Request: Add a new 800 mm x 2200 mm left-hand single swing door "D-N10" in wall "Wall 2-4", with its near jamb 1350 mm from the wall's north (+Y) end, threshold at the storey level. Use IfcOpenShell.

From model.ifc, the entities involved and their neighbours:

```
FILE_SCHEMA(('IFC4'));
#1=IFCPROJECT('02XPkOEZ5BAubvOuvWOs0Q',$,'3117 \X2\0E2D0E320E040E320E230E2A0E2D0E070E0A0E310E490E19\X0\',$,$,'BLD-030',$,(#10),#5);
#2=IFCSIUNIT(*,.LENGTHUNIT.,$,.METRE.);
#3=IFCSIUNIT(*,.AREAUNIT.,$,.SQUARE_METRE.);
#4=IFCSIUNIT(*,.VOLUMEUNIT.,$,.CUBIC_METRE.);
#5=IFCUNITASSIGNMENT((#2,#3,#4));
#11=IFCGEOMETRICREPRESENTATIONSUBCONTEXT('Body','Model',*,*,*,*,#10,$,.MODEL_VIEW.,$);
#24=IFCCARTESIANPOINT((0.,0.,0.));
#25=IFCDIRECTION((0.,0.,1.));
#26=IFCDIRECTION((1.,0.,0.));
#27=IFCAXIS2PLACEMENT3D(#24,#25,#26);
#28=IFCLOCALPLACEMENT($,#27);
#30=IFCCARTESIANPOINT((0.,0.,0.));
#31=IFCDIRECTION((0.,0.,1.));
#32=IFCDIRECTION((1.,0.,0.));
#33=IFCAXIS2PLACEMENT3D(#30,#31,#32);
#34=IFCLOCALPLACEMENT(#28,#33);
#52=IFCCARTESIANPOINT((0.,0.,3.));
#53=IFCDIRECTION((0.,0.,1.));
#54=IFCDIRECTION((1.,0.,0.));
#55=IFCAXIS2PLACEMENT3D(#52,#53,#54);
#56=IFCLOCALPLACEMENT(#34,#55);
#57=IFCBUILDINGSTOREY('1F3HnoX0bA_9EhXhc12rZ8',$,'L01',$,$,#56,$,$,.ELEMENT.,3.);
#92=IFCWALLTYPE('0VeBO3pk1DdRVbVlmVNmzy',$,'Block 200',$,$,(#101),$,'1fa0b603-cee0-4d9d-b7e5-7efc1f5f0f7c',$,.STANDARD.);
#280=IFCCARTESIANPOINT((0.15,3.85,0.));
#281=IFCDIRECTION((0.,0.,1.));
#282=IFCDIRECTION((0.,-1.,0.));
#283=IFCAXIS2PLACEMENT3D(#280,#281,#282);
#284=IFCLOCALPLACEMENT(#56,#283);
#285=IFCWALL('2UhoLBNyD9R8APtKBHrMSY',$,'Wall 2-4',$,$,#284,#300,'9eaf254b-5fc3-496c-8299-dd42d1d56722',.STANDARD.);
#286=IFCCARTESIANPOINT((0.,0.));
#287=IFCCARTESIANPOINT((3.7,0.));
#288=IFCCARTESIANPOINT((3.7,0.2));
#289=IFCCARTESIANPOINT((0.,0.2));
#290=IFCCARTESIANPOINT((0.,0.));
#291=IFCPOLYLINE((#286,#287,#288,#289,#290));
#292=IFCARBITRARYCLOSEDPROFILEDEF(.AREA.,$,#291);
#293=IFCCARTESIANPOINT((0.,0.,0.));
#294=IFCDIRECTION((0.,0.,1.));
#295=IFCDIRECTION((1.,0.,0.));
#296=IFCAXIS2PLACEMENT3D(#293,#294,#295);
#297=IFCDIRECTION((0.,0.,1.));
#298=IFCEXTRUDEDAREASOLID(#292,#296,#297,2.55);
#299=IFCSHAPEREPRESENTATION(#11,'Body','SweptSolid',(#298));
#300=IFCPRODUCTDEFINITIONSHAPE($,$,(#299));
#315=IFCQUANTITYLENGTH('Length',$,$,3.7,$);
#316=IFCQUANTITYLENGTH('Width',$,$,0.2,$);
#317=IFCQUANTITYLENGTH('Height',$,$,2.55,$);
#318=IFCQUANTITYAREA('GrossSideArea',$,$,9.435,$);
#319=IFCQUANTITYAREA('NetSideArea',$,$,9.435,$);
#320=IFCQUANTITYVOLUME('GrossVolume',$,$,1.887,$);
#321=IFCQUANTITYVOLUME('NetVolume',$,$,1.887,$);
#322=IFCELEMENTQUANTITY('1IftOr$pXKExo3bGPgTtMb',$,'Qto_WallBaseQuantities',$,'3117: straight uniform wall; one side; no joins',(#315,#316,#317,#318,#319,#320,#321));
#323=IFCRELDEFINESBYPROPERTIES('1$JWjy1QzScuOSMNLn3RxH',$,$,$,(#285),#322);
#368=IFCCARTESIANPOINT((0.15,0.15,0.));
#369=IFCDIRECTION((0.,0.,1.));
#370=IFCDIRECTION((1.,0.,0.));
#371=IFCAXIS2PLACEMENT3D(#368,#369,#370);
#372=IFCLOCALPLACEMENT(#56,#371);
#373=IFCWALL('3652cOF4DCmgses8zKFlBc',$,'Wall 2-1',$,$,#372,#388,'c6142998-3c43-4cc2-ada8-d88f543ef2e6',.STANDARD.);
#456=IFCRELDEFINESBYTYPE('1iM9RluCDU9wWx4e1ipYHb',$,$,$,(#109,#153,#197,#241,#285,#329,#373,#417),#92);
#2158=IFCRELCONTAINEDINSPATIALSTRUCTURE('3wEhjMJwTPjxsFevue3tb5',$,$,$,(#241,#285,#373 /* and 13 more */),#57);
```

```python
import numpy as np
import ifcopenshell
import ifcopenshell.api.feature
import ifcopenshell.api.geometry
import ifcopenshell.api.pset
import ifcopenshell.api.root
import ifcopenshell.api.spatial
import ifcopenshell.geom
import ifcopenshell.util.element
import ifcopenshell.util.placement
import ifcopenshell.util.representation
import ifcopenshell.util.shape
import ifcopenshell.util.unit

model = ifcopenshell.open("model.ifc")
unit_scale = ifcopenshell.util.unit.calculate_unit_scale(model)
area_scale = ifcopenshell.util.unit.calculate_unit_scale(model, "AREAUNIT")
volume_scale = ifcopenshell.util.unit.calculate_unit_scale(model, "VOLUMEUNIT")
settings = ifcopenshell.geom.settings()


def volume(element):
    """Net volume in cubic metres, openings subtracted."""
    shape = ifcopenshell.geom.create_shape(settings, element)
    return ifcopenshell.util.shape.get_volume(shape.geometry)


wall = model.by_guid("2UhoLBNyD9R8APtKBHrMSY")
storey = ifcopenshell.util.element.get_container(wall, ifc_class="IfcBuildingStorey")
context = ifcopenshell.util.representation.get_context(model, "Model", "Body", "MODEL_VIEW")
before = volume(wall)

width, height, from_end, sill = 0.8, 2.2, 1.35, 0.0  # metres

# The wall runs along its own X axis, and the end named is its -X end.
wall_shape = ifcopenshell.geom.create_shape(settings, wall)
x, y, z = ifcopenshell.util.shape.get_vertices(wall_shape.geometry).T
start = x.min() + from_end
face, thickness = float(y.min()), float(y.max() - y.min())
wall_matrix = ifcopenshell.util.placement.get_local_placement(wall.ObjectPlacement)
level = ifcopenshell.util.placement.get_local_placement(storey.ObjectPlacement)[2, 3]


def in_wall(x, y):
    """Placement at x, y metres in the wall's axes, at sill height."""
    matrix = wall_matrix.copy()
    matrix[:, 3] = wall_matrix @ np.array([x / unit_scale, y / unit_scale, 0.0, 1.0])
    matrix[2, 3] = level + sill / unit_scale
    return matrix


# Opening: a box that overshoots both wall faces by 50 mm.
opening = ifcopenshell.api.root.create_entity(model, ifc_class="IfcOpeningElement", predefined_type="OPENING")
box = ifcopenshell.api.geometry.add_wall_representation(
    model, context=context, length=width, height=height, thickness=thickness + 0.1
)
ifcopenshell.api.geometry.assign_representation(model, product=opening, representation=box)
ifcopenshell.api.geometry.edit_object_placement(model, product=opening, matrix=in_wall(start, face - 0.05), is_si=False)
ifcopenshell.api.feature.add_feature(model, feature=opening, element=wall)

door = ifcopenshell.api.root.create_entity(model, ifc_class="IfcDoor", name="D-N10", predefined_type="DOOR")
door.OverallWidth, door.OverallHeight = width / unit_scale, height / unit_scale
door.OperationType = "SINGLE_SWING_LEFT"
body = ifcopenshell.api.geometry.add_door_representation(
    model,
    context=context,
    overall_width=door.OverallWidth,
    overall_height=door.OverallHeight,
    operation_type="SINGLE_SWING_LEFT",
    lining_properties={"LiningDepth": thickness / unit_scale, "ThresholdDepth": thickness / unit_scale},
)
ifcopenshell.api.geometry.assign_representation(model, product=door, representation=body)
ifcopenshell.api.spatial.assign_container(model, products=[door], relating_structure=storey)
ifcopenshell.api.feature.add_filling(model, opening=opening, element=door)

# The lining spans the wall, so the door starts at the wall face.
ifcopenshell.api.geometry.edit_object_placement(model, product=door, matrix=in_wall(start, face), is_si=False)

after = volume(wall)

# Update the wall's stored quantities.
qto = model.by_id(ifcopenshell.util.element.get_pset(wall, "Qto_WallBaseQuantities", should_inherit=False)["id"])
ifcopenshell.api.pset.edit_qto(model, qto=qto, properties={
    "NetSideArea": after / thickness / area_scale,
    "NetVolume": after / volume_scale,
})

print(f"wall volume {before:.3f} -> {after:.3f} m3")

model.write("model_updated.ifc")
```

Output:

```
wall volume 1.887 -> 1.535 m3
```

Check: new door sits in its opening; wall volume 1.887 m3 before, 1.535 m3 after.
